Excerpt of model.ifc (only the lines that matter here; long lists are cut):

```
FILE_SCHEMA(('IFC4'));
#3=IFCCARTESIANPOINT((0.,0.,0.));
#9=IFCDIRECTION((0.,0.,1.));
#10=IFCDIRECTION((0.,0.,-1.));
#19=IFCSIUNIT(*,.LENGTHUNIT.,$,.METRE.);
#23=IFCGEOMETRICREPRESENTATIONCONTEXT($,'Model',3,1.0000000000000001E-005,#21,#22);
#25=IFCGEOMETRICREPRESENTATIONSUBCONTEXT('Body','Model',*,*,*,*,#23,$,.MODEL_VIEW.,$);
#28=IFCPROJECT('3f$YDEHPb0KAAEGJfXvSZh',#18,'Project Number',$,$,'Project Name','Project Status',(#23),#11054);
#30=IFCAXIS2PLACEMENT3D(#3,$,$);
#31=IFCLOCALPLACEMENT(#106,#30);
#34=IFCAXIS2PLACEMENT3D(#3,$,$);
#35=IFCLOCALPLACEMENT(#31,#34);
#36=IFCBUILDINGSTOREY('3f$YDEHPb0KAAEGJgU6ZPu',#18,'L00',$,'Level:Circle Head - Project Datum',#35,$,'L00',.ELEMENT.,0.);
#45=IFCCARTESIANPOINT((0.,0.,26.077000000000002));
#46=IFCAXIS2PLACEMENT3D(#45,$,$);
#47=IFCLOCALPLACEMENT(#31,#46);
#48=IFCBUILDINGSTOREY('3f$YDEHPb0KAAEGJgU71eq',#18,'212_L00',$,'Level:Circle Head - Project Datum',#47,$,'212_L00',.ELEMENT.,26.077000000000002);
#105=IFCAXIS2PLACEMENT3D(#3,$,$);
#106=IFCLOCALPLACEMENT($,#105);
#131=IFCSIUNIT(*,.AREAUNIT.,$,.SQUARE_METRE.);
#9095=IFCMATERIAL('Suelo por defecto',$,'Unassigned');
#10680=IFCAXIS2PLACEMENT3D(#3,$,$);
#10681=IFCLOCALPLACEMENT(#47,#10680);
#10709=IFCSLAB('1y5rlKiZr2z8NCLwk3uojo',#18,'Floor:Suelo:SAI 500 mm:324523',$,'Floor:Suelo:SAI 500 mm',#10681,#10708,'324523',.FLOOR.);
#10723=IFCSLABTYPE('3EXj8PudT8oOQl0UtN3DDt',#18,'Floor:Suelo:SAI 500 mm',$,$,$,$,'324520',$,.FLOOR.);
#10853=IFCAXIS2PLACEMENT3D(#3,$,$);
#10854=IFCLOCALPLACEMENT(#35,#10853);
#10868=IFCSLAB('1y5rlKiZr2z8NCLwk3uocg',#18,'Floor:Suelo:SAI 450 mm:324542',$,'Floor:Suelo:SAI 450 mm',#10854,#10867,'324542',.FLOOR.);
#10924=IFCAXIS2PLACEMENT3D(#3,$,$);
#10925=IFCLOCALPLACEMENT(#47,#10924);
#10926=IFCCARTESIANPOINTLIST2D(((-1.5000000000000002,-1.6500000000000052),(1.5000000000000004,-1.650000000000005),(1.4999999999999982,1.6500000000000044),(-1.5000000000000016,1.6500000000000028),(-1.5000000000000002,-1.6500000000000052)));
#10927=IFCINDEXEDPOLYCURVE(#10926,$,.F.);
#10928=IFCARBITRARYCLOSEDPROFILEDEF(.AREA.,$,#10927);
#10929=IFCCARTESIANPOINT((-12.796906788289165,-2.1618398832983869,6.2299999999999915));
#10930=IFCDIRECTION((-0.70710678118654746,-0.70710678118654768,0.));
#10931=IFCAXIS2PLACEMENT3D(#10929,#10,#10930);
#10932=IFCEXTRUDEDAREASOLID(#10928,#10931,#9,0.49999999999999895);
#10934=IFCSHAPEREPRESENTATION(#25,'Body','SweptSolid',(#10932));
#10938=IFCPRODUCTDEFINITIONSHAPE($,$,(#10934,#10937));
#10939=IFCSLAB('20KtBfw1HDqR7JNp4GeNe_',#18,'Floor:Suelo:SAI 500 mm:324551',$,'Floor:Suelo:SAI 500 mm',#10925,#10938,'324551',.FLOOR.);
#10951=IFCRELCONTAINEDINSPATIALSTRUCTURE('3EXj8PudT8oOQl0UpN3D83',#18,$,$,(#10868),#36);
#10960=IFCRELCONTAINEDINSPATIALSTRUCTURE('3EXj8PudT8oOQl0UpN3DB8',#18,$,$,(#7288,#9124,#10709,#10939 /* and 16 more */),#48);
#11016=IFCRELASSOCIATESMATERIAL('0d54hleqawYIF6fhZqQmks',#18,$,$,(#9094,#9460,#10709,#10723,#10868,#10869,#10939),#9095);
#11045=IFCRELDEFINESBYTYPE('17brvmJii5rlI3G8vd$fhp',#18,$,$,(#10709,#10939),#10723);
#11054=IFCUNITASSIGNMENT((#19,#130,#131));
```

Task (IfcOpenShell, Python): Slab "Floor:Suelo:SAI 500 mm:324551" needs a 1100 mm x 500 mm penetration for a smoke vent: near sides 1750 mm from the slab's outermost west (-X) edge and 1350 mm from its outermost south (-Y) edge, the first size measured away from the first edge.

```python
import numpy as np
import ifcopenshell
import ifcopenshell.api.feature
import ifcopenshell.api.geometry
import ifcopenshell.api.root
import ifcopenshell.geom
import ifcopenshell.util.placement
import ifcopenshell.util.representation
import ifcopenshell.util.shape
import ifcopenshell.util.unit

model = ifcopenshell.open("model.ifc")
unit_scale = ifcopenshell.util.unit.calculate_unit_scale(model)
settings = ifcopenshell.geom.settings()


def volume(element):
    """Net volume in cubic metres, openings subtracted."""
    shape = ifcopenshell.geom.create_shape(settings, element)
    return ifcopenshell.util.shape.get_volume(shape.geometry)


slab = model.by_guid("20KtBfw1HDqR7JNp4GeNe_")
before = volume(slab)

# Extent in the slab's own axes, in metres. The edges named are its -X and -Y sides.
slab_shape = ifcopenshell.geom.create_shape(settings, slab)
vertices = ifcopenshell.util.shape.get_vertices(slab_shape.geometry)
x_min, y_min, bottom = vertices.min(axis=0)
top = vertices[:, 2].max()

opening = ifcopenshell.api.root.create_entity(model, ifc_class="IfcOpeningElement", name="Smoke vent opening", predefined_type="OPENING")
context = ifcopenshell.util.representation.get_context(model, "Model", "Body", "MODEL_VIEW")
width, depth = 1.1, 0.5
outline = [(0.0, 0.0), (width, 0.0), (width, depth), (0.0, depth), (0.0, 0.0)]
# Overshoot both faces by 50 mm so the cut is clean.
shape = ifcopenshell.api.geometry.add_slab_representation(
    model, context=context, depth=top - bottom + 0.1, polyline=outline
)
ifcopenshell.api.geometry.assign_representation(model, product=opening, representation=shape)

matrix = ifcopenshell.util.placement.get_local_placement(slab.ObjectPlacement)
matrix[:, 3] = matrix @ np.append(np.array([x_min + 1.75, y_min + 1.35, bottom - 0.05]) / unit_scale, 1.0)
ifcopenshell.api.geometry.edit_object_placement(model, product=opening, matrix=matrix, is_si=False)
ifcopenshell.api.feature.add_feature(model, feature=opening, element=slab)

after = volume(slab)

print(f"slab volume {before:.3f} -> {after:.3f} m3")

model.write("model_v2.ifc")
```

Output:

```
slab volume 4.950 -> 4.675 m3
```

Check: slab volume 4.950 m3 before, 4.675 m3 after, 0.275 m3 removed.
